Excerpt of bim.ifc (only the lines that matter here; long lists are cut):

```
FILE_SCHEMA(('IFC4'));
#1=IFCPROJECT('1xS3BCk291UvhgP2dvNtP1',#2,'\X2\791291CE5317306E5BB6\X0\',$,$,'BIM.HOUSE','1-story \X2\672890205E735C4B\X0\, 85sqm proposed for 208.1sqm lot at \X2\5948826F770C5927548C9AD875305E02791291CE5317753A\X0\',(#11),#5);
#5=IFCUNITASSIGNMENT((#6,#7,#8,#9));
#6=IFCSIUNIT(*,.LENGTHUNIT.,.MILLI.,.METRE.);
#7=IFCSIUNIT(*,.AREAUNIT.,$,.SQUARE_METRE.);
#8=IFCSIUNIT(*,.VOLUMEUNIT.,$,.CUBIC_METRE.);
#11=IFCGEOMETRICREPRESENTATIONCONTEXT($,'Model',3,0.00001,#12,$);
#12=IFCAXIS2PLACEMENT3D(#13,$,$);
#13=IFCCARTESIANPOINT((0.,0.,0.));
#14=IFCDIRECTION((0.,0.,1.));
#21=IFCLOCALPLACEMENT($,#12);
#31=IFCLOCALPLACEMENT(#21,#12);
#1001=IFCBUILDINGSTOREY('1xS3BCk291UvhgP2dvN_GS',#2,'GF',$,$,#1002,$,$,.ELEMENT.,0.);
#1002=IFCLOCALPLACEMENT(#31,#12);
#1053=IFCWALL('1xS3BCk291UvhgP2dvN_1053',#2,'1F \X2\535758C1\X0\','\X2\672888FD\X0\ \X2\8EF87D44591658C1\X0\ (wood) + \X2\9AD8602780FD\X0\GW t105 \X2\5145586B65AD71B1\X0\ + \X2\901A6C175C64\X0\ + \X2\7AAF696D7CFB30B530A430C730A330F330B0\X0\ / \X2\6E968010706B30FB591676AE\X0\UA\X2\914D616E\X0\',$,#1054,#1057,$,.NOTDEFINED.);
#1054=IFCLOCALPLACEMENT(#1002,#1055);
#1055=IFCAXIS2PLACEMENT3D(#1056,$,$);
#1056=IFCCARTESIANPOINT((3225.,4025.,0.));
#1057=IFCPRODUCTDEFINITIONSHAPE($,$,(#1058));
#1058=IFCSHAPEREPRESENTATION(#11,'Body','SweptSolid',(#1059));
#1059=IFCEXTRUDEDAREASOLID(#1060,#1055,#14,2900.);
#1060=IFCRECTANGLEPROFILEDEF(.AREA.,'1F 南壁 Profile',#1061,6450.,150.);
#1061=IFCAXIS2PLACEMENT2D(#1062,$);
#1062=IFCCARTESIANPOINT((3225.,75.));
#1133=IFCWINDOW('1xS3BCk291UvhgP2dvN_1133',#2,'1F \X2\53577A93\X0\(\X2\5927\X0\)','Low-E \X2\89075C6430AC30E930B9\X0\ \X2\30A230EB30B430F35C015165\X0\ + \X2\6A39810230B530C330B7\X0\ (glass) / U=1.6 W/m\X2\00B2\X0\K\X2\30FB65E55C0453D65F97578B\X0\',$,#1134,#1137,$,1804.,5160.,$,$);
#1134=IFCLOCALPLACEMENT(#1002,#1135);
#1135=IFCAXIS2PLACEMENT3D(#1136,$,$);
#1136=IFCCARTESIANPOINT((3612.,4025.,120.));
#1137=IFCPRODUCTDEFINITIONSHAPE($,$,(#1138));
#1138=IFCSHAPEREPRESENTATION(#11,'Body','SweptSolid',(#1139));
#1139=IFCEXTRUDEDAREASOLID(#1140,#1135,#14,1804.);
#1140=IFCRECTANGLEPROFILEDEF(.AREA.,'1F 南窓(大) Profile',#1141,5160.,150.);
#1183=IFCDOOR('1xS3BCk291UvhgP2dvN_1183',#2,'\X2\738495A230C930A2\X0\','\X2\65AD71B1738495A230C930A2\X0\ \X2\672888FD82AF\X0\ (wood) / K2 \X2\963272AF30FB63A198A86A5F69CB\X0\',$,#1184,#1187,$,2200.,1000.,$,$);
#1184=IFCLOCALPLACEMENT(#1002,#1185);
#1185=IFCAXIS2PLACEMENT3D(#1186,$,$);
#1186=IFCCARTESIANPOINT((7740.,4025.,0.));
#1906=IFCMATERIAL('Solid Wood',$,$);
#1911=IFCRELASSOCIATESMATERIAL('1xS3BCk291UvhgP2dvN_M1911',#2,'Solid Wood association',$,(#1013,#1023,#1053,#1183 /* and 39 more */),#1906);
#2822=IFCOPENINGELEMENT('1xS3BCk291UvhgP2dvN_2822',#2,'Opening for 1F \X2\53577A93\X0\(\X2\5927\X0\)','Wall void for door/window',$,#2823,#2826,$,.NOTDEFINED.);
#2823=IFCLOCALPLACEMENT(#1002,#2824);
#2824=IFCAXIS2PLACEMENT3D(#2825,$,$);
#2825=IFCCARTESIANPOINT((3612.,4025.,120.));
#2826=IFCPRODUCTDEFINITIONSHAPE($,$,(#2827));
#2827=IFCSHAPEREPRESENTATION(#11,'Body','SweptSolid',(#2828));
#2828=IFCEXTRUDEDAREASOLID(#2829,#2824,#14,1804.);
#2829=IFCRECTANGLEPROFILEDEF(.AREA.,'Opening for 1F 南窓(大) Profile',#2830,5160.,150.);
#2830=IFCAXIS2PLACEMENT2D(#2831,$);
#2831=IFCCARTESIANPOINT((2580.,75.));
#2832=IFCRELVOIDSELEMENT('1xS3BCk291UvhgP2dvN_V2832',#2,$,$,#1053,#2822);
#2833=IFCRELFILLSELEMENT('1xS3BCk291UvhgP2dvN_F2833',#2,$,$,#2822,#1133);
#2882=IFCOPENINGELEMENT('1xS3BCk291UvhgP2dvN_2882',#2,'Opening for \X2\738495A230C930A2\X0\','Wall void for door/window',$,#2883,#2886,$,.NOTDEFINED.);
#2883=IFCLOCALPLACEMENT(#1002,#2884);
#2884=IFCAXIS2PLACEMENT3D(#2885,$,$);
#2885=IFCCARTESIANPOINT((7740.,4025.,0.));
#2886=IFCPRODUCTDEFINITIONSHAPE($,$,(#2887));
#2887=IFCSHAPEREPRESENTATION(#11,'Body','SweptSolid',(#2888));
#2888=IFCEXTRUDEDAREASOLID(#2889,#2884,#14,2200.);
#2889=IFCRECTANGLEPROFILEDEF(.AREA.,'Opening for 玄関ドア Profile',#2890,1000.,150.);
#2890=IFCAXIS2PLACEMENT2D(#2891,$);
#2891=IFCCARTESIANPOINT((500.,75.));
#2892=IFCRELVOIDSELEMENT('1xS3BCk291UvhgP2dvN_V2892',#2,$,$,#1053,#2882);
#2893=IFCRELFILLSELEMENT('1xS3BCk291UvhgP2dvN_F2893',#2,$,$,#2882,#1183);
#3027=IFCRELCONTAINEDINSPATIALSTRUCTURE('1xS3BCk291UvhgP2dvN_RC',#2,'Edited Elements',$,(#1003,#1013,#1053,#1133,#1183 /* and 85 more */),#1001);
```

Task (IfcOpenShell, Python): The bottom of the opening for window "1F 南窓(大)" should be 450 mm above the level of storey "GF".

```python
import numpy as np
import ifcopenshell
import ifcopenshell.api.geometry
import ifcopenshell.geom
import ifcopenshell.util.element
import ifcopenshell.util.placement
import ifcopenshell.util.shape
import ifcopenshell.util.unit

model = ifcopenshell.open("bim.ifc")
unit_scale = ifcopenshell.util.unit.calculate_unit_scale(model)

window = model.by_id(1133)
opening = window.FillsVoids[0].RelatingOpeningElement
storey = ifcopenshell.util.element.get_container(window, ifc_class="IfcBuildingStorey")
level = ifcopenshell.util.placement.get_local_placement(storey.ObjectPlacement)[2, 3]

# The opening's origin need not be at the sill, so measure its lowest point.
shape = ifcopenshell.geom.create_shape(ifcopenshell.geom.settings(), opening)
bottom = ifcopenshell.util.shape.get_shape_bottom_elevation(shape, shape.geometry) / unit_scale
dz = level + 0.45 / unit_scale - bottom

shift = np.array([0.0, 0.0, dz])
# The window is not placed relative to its opening, so move both.
for product in (opening, window):
    matrix = ifcopenshell.util.placement.get_local_placement(product.ObjectPlacement)
    matrix[:3, 3] += shift
    ifcopenshell.api.geometry.edit_object_placement(model, product=product, matrix=matrix, is_si=False)

print(f"moved by {dz * unit_scale:+.3f} m")

model.write("bim_edited.ifc")
```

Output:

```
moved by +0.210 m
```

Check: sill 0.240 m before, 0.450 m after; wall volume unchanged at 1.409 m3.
